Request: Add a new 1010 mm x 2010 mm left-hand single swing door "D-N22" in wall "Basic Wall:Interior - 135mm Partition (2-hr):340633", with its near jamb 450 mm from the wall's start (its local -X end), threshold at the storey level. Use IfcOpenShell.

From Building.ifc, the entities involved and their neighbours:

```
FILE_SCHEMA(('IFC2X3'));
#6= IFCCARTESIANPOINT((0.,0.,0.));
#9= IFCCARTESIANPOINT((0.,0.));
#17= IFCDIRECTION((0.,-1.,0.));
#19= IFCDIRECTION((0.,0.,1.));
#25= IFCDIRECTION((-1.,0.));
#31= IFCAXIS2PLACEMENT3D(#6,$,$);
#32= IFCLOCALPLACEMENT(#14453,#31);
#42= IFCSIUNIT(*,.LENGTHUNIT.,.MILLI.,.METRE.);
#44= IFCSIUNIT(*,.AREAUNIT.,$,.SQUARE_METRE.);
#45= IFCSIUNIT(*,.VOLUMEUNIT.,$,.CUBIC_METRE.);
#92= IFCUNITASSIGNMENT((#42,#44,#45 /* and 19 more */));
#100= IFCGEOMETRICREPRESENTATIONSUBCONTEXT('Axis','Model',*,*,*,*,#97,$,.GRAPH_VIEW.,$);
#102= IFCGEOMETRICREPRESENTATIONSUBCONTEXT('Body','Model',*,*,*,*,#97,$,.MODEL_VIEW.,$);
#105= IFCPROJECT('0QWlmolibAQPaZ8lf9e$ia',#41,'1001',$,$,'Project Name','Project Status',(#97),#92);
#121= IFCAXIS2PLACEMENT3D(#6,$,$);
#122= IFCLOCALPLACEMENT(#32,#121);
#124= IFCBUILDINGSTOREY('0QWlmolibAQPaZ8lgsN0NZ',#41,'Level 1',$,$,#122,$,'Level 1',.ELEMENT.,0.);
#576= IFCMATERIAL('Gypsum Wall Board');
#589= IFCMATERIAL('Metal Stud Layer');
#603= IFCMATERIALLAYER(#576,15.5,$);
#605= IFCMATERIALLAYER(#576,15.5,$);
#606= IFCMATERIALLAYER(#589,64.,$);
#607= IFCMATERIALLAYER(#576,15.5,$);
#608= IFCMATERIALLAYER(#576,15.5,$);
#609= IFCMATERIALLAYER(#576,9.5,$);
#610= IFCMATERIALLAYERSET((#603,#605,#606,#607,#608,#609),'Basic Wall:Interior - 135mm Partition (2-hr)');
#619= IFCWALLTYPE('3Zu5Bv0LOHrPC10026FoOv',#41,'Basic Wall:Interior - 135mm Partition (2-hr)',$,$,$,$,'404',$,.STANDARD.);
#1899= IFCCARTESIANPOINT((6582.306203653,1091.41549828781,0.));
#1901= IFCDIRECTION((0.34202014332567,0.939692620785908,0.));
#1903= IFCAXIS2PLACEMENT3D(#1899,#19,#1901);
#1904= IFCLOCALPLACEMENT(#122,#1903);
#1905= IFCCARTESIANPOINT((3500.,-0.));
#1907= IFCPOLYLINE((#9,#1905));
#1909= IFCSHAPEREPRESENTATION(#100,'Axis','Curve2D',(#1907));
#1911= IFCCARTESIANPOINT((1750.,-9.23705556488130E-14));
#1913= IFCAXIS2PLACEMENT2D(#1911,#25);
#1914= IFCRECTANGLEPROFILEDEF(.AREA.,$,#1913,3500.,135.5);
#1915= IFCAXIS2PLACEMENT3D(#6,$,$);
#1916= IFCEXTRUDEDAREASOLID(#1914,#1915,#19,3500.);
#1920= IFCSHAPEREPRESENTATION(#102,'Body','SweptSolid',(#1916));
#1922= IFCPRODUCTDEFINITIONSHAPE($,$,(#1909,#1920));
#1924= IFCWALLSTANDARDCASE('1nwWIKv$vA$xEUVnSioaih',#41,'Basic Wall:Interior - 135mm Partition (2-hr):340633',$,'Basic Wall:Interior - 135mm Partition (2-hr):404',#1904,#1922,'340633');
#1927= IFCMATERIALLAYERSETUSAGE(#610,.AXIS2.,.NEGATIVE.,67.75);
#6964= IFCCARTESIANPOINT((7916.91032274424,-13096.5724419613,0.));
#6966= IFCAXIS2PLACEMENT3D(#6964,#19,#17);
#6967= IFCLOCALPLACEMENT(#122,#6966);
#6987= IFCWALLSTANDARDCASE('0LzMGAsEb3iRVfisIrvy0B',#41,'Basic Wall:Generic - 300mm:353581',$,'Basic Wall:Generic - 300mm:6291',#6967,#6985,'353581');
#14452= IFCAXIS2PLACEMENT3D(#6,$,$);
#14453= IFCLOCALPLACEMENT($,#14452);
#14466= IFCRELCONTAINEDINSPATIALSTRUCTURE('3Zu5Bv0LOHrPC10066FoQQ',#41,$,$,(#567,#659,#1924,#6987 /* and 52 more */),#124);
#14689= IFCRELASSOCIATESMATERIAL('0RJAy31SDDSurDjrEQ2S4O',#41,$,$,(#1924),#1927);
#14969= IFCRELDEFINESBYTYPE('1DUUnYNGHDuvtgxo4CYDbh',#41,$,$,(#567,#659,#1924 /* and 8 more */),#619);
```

```python
import numpy as np
import ifcopenshell
import ifcopenshell.api.feature
import ifcopenshell.api.geometry
import ifcopenshell.api.root
import ifcopenshell.api.spatial
import ifcopenshell.api.type
import ifcopenshell.geom
import ifcopenshell.util.element
import ifcopenshell.util.placement
import ifcopenshell.util.representation
import ifcopenshell.util.shape
import ifcopenshell.util.unit

model = ifcopenshell.open("Building.ifc")
unit_scale = ifcopenshell.util.unit.calculate_unit_scale(model)
settings = ifcopenshell.geom.settings()


def volume(element):
    """Net volume in cubic metres, openings subtracted."""
    shape = ifcopenshell.geom.create_shape(settings, element)
    return ifcopenshell.util.shape.get_volume(shape.geometry)


wall = model.by_id(1924)
storey = ifcopenshell.util.element.get_container(wall, ifc_class="IfcBuildingStorey")
context = ifcopenshell.util.representation.get_context(model, "Model", "Body", "MODEL_VIEW")
before = volume(wall)

width, height, from_end, sill = 1.01, 2.01, 0.45, 0.0  # metres

# The wall runs along its own X axis, and the end named is its -X end.
wall_shape = ifcopenshell.geom.create_shape(settings, wall)
x, y, z = ifcopenshell.util.shape.get_vertices(wall_shape.geometry).T
start = x.min() + from_end
face, thickness = float(y.min()), float(y.max() - y.min())
wall_matrix = ifcopenshell.util.placement.get_local_placement(wall.ObjectPlacement)
level = ifcopenshell.util.placement.get_local_placement(storey.ObjectPlacement)[2, 3]


def in_wall(x, y):
    """Placement at x, y metres in the wall's axes, at sill height."""
    matrix = wall_matrix.copy()
    matrix[:, 3] = wall_matrix @ np.array([x / unit_scale, y / unit_scale, 0.0, 1.0])
    matrix[2, 3] = level + sill / unit_scale
    return matrix


# Opening: a box that overshoots both wall faces by 50 mm.
opening = ifcopenshell.api.root.create_entity(model, ifc_class="IfcOpeningElement")
box = ifcopenshell.api.geometry.add_wall_representation(
    model, context=context, length=width, height=height, thickness=thickness + 0.1
)
ifcopenshell.api.geometry.assign_representation(model, product=opening, representation=box)
ifcopenshell.api.geometry.edit_object_placement(model, product=opening, matrix=in_wall(start, face - 0.05), is_si=False)
ifcopenshell.api.feature.add_feature(model, feature=opening, element=wall)

door = ifcopenshell.api.root.create_entity(model, ifc_class="IfcDoor", name="D-N22")
door.OverallWidth, door.OverallHeight = width / unit_scale, height / unit_scale
body = ifcopenshell.api.geometry.add_door_representation(
    model,
    context=context,
    overall_width=door.OverallWidth,
    overall_height=door.OverallHeight,
    operation_type="SINGLE_SWING_LEFT",
    lining_properties={"LiningDepth": thickness / unit_scale, "ThresholdDepth": thickness / unit_scale},
)
ifcopenshell.api.geometry.assign_representation(model, product=door, representation=body)
ifcopenshell.api.spatial.assign_container(model, products=[door], relating_structure=storey)
fills = ifcopenshell.api.feature.add_filling(model, opening=opening, element=door)
fills.OwnerHistory = door.OwnerHistory  # required in IFC2X3

# IFC2X3 keeps the operation on the door style.
style = ifcopenshell.api.root.create_entity(model, ifc_class="IfcDoorStyle", name="D-N22")
style.OperationType, style.ConstructionType = "SINGLE_SWING_LEFT", "NOTDEFINED"
style.ParameterTakesPrecedence = style.Sizeable = False
ifcopenshell.api.type.assign_type(model, related_objects=[door], relating_type=style)

# The lining spans the wall, so the door starts at the wall face.
ifcopenshell.api.geometry.edit_object_placement(model, product=door, matrix=in_wall(start, face), is_si=False)

after = volume(wall)

print(f"wall volume {before:.3f} -> {after:.3f} m3")

model.write("Building_edited.ifc")
```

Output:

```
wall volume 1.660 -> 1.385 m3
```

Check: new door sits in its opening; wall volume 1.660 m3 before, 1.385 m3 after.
